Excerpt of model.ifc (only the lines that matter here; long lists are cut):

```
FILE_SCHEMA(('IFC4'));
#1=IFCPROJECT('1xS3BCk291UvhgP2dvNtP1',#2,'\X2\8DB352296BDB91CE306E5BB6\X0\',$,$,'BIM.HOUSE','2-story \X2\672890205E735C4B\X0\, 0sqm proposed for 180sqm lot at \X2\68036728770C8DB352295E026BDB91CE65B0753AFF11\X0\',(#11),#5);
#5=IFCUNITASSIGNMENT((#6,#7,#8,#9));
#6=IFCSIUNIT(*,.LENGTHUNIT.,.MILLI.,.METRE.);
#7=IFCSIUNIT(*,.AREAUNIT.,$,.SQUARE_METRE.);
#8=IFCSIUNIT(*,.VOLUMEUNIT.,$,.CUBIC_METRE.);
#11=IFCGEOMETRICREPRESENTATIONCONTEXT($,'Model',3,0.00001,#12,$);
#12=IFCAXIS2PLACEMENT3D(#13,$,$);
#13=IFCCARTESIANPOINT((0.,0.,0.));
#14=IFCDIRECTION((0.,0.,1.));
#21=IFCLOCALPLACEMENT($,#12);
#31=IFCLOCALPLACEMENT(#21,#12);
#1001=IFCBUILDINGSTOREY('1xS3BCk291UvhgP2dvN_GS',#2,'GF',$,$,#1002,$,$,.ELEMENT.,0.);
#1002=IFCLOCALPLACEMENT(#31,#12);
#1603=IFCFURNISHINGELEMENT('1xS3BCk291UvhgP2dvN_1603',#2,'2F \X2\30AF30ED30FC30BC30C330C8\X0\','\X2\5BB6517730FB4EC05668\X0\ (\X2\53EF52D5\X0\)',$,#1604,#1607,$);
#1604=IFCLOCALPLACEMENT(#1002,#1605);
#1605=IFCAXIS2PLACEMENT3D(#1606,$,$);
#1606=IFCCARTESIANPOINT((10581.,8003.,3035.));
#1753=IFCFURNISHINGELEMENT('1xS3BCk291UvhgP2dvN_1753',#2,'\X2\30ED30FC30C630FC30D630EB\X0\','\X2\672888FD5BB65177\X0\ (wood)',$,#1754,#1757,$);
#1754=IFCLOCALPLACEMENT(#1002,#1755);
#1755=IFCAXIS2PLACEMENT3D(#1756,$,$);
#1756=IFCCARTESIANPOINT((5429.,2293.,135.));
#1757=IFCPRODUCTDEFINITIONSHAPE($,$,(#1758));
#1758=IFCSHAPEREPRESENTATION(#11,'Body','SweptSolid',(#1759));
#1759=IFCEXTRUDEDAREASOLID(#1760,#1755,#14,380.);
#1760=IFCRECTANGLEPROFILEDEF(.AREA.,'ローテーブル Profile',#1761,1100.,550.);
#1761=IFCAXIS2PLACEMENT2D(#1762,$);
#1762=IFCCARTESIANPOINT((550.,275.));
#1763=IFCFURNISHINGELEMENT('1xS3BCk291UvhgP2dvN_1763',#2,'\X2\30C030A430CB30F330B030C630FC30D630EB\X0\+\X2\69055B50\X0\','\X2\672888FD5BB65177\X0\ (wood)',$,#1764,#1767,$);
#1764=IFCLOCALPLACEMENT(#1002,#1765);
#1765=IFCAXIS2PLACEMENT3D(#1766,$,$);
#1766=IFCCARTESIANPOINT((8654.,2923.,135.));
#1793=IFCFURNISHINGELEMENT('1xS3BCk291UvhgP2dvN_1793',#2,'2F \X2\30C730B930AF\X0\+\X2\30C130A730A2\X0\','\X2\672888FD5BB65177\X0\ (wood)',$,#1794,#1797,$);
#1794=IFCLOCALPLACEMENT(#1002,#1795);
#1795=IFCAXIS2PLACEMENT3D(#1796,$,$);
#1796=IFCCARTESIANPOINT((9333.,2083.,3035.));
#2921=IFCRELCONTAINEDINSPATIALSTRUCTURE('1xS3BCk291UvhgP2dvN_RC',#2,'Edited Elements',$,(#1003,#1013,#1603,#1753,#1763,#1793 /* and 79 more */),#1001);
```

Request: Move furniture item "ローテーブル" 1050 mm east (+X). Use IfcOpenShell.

```python
import ifcopenshell
import ifcopenshell.api.geometry
import ifcopenshell.util.placement

model = ifcopenshell.open("model.ifc")

item = model.by_id(1753)
matrix = ifcopenshell.util.placement.get_local_placement(item.ObjectPlacement)
matrix[0, 3] += 1050.0
ifcopenshell.api.geometry.edit_object_placement(model, product=item, matrix=matrix, is_si=False)

print(ifcopenshell.util.placement.get_local_placement(item.ObjectPlacement).round(3) + 0.0)

model.write("model_updated.ifc")
```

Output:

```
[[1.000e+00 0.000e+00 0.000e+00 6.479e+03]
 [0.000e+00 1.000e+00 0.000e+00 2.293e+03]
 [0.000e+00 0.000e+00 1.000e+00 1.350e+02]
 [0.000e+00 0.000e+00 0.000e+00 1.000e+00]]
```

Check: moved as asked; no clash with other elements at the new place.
